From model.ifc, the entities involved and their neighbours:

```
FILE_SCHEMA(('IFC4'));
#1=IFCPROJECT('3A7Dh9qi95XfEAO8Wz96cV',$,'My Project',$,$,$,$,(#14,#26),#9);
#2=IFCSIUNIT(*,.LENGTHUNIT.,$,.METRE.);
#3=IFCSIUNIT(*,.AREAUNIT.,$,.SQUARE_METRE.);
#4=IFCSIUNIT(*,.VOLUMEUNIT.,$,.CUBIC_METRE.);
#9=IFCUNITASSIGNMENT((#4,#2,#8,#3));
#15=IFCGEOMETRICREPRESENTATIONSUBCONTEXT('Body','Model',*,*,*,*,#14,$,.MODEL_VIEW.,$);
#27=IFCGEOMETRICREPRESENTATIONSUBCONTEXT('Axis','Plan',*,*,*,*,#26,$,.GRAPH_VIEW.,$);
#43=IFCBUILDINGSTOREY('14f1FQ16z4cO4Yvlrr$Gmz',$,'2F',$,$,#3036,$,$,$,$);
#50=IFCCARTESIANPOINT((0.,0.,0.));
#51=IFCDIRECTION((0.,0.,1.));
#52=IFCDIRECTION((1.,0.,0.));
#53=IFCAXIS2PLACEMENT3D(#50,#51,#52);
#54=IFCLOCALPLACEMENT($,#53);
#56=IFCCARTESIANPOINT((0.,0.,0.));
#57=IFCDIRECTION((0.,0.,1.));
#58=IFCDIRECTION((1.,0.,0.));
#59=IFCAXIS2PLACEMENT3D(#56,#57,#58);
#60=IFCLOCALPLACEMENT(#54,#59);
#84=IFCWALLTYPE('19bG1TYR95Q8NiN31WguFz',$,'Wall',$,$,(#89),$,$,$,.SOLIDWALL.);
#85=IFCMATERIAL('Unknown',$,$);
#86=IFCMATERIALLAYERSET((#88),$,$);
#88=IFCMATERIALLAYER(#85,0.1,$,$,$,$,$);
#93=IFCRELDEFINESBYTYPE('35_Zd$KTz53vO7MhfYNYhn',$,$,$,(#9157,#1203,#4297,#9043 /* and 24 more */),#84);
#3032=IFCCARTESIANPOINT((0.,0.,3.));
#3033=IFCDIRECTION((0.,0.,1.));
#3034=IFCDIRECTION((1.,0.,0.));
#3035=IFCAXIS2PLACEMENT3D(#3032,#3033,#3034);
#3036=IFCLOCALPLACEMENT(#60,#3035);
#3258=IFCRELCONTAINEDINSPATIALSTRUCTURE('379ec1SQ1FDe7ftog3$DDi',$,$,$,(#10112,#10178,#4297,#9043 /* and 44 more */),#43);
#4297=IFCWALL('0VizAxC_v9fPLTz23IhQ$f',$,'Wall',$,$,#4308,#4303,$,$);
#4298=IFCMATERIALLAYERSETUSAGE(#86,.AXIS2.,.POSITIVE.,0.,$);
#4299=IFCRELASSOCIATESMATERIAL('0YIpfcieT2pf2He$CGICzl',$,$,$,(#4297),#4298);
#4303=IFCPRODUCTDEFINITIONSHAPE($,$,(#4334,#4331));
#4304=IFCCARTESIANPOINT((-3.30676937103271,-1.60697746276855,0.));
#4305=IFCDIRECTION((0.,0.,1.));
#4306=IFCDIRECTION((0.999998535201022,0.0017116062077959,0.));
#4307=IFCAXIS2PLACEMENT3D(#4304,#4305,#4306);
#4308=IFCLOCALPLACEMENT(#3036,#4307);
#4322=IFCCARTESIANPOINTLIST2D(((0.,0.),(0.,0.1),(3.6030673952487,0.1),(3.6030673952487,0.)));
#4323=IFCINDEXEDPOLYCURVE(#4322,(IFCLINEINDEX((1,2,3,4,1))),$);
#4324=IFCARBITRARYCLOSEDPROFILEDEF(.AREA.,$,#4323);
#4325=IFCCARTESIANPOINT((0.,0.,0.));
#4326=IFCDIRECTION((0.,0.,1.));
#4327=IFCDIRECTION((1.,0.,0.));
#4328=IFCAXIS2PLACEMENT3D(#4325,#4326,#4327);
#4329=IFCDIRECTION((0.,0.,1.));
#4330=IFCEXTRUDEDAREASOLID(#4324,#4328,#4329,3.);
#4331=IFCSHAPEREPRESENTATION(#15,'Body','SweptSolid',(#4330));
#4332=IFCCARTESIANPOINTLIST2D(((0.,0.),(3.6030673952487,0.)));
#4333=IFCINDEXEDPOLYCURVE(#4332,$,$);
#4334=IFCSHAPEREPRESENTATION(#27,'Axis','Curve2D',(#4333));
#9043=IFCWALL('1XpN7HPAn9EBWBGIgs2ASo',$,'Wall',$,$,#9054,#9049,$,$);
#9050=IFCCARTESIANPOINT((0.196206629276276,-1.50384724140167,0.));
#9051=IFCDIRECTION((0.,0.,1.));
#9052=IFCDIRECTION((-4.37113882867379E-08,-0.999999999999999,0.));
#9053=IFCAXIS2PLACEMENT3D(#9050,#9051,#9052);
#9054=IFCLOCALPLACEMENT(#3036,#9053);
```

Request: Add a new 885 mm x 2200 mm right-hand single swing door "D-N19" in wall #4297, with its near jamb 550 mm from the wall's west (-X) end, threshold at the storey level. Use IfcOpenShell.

```python
import numpy as np
import ifcopenshell
import ifcopenshell.api.feature
import ifcopenshell.api.geometry
import ifcopenshell.api.root
import ifcopenshell.api.spatial
import ifcopenshell.geom
import ifcopenshell.util.element
import ifcopenshell.util.placement
import ifcopenshell.util.representation
import ifcopenshell.util.shape
import ifcopenshell.util.unit

model = ifcopenshell.open("model.ifc")
unit_scale = ifcopenshell.util.unit.calculate_unit_scale(model)
settings = ifcopenshell.geom.settings()


def volume(element):
    """Net volume in cubic metres, openings subtracted."""
    shape = ifcopenshell.geom.create_shape(settings, element)
    return ifcopenshell.util.shape.get_volume(shape.geometry)


wall = model.by_guid("0VizAxC_v9fPLTz23IhQ$f")
storey = ifcopenshell.util.element.get_container(wall, ifc_class="IfcBuildingStorey")
context = ifcopenshell.util.representation.get_context(model, "Model", "Body", "MODEL_VIEW")
before = volume(wall)

width, height, from_end, sill = 0.885, 2.2, 0.55, 0.0  # metres

# The wall runs along its own X axis, and the end named is its -X end.
wall_shape = ifcopenshell.geom.create_shape(settings, wall)
x, y, z = ifcopenshell.util.shape.get_vertices(wall_shape.geometry).T
start = x.min() + from_end
face, thickness = float(y.min()), float(y.max() - y.min())
wall_matrix = ifcopenshell.util.placement.get_local_placement(wall.ObjectPlacement)
level = ifcopenshell.util.placement.get_local_placement(storey.ObjectPlacement)[2, 3]


def in_wall(x, y):
    """Placement at x, y metres in the wall's axes, at sill height."""
    matrix = wall_matrix.copy()
    matrix[:, 3] = wall_matrix @ np.array([x / unit_scale, y / unit_scale, 0.0, 1.0])
    matrix[2, 3] = level + sill / unit_scale
    return matrix


# Opening: a box that overshoots both wall faces by 50 mm.
opening = ifcopenshell.api.root.create_entity(model, ifc_class="IfcOpeningElement", predefined_type="OPENING")
box = ifcopenshell.api.geometry.add_wall_representation(
    model, context=context, length=width, height=height, thickness=thickness + 0.1
)
ifcopenshell.api.geometry.assign_representation(model, product=opening, representation=box)
ifcopenshell.api.geometry.edit_object_placement(model, product=opening, matrix=in_wall(start, face - 0.05), is_si=False)
ifcopenshell.api.feature.add_feature(model, feature=opening, element=wall)

door = ifcopenshell.api.root.create_entity(model, ifc_class="IfcDoor", name="D-N19", predefined_type="DOOR")
door.OverallWidth, door.OverallHeight = width / unit_scale, height / unit_scale
door.OperationType = "SINGLE_SWING_RIGHT"
body = ifcopenshell.api.geometry.add_door_representation(
    model,
    context=context,
    overall_width=door.OverallWidth,
    overall_height=door.OverallHeight,
    operation_type="SINGLE_SWING_RIGHT",
    lining_properties={"LiningDepth": thickness / unit_scale, "ThresholdDepth": thickness / unit_scale},
)
ifcopenshell.api.geometry.assign_representation(model, product=door, representation=body)
ifcopenshell.api.spatial.assign_container(model, products=[door], relating_structure=storey)
ifcopenshell.api.feature.add_filling(model, opening=opening, element=door)

# The lining spans the wall, so the door starts at the wall face.
ifcopenshell.api.geometry.edit_object_placement(model, product=door, matrix=in_wall(start, face), is_si=False)

after = volume(wall)

print(f"wall volume {before:.3f} -> {after:.3f} m3")

model.write("model_rev.ifc")
```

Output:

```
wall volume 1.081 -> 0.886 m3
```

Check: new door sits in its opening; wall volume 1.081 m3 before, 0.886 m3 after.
